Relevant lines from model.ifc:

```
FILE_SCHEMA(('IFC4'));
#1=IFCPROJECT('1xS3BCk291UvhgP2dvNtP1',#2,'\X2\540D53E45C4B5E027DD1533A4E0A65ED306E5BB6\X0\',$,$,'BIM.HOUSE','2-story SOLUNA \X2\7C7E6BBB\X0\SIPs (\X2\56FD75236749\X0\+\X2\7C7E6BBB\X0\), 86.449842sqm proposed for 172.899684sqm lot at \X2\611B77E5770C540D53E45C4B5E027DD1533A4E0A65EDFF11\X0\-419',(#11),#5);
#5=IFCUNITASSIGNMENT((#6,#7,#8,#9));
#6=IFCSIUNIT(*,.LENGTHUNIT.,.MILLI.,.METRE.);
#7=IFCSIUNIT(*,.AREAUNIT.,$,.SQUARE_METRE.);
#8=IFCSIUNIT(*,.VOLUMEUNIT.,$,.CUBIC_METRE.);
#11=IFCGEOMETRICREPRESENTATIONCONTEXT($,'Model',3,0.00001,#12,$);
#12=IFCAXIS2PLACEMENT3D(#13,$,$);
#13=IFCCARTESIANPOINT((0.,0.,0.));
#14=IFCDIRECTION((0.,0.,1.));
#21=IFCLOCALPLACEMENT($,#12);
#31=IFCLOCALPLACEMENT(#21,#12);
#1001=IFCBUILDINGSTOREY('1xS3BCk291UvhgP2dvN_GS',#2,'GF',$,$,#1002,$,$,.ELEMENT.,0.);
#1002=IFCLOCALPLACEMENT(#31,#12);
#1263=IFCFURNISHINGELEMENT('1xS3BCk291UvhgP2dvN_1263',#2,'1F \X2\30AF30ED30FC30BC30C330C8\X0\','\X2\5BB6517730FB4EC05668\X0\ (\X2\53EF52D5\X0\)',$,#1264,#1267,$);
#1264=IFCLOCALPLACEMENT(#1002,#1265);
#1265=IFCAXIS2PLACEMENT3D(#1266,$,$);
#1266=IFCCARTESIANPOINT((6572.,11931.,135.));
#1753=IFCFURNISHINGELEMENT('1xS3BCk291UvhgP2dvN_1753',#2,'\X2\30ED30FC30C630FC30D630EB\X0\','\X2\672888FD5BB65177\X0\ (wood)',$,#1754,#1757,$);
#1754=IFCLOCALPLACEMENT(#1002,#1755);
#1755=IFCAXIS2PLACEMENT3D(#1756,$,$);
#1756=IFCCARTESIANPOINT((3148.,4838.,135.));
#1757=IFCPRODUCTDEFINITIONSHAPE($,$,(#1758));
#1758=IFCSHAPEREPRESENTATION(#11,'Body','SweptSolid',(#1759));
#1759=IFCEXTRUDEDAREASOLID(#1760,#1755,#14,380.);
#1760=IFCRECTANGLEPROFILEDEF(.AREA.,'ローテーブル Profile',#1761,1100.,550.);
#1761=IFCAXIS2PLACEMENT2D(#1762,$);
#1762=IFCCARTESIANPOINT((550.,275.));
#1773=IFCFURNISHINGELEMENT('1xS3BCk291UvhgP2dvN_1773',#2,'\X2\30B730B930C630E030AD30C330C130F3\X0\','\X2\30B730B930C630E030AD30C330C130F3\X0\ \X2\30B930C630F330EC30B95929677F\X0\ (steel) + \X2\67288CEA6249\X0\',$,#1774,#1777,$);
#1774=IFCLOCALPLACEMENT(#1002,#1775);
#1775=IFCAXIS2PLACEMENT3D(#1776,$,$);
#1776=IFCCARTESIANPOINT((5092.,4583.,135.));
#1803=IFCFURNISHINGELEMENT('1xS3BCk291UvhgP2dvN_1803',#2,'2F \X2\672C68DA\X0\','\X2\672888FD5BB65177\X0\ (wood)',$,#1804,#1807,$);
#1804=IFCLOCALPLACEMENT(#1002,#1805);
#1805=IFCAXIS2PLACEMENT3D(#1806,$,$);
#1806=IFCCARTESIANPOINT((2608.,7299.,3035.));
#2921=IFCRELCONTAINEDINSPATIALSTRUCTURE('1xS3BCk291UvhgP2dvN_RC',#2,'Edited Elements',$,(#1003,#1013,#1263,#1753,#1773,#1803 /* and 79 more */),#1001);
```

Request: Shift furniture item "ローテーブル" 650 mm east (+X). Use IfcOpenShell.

```python
import ifcopenshell
import ifcopenshell.api.geometry
import ifcopenshell.util.placement

model = ifcopenshell.open("model.ifc")

item = model.by_guid("1xS3BCk291UvhgP2dvN_1753")
matrix = ifcopenshell.util.placement.get_local_placement(item.ObjectPlacement)
matrix[0, 3] += 650.0
ifcopenshell.api.geometry.edit_object_placement(model, product=item, matrix=matrix, is_si=False)

print(ifcopenshell.util.placement.get_local_placement(item.ObjectPlacement).round(3) + 0.0)

model.write("model_edited.ifc")
```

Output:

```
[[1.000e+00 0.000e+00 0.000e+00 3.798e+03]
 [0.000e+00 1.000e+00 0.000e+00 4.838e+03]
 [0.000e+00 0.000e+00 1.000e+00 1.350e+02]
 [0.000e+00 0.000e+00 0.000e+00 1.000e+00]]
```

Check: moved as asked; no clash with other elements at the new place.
